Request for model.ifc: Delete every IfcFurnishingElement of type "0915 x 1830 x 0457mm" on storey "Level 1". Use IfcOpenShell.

First a look at what the model holds.

```python
import ifcopenshell
import ifcopenshell.util.element

model = ifcopenshell.open("model.ifc")
print(model.schema)
storey = next(s for s in model.by_type("IfcBuildingStorey") if s.Name == "Level 1")
furniture = [e for e in ifcopenshell.util.element.get_decomposition(storey) if e.is_a("IfcFurnishingElement")]
seen = {}
for e in furniture:
    element_type = ifcopenshell.util.element.get_type(e)
    name = element_type.Name if element_type not in (None, e) else None
    seen[name] = seen.get(name, 0) + 1
for name, count in sorted(seen.items(), key=str):
    print(count, "x", name)
```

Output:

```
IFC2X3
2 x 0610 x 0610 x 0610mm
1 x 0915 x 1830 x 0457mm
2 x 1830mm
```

```python
import ifcopenshell
import ifcopenshell.api.root
import ifcopenshell.util.element

model = ifcopenshell.open("model.ifc")

storey = next(s for s in model.by_type("IfcBuildingStorey") if s.Name == "Level 1")
furniture = [e for e in ifcopenshell.util.element.get_decomposition(storey) if e.is_a("IfcFurnishingElement")]
targets = [e for e in furniture if (t := ifcopenshell.util.element.get_type(e)) not in (None, e) and t.Name == "0915 x 1830 x 0457mm"]

for e in targets:
    ifcopenshell.api.root.remove_product(model, product=e)
print(len(targets), "removed")

model.write("model_edited.ifc")
```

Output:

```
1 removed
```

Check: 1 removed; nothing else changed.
